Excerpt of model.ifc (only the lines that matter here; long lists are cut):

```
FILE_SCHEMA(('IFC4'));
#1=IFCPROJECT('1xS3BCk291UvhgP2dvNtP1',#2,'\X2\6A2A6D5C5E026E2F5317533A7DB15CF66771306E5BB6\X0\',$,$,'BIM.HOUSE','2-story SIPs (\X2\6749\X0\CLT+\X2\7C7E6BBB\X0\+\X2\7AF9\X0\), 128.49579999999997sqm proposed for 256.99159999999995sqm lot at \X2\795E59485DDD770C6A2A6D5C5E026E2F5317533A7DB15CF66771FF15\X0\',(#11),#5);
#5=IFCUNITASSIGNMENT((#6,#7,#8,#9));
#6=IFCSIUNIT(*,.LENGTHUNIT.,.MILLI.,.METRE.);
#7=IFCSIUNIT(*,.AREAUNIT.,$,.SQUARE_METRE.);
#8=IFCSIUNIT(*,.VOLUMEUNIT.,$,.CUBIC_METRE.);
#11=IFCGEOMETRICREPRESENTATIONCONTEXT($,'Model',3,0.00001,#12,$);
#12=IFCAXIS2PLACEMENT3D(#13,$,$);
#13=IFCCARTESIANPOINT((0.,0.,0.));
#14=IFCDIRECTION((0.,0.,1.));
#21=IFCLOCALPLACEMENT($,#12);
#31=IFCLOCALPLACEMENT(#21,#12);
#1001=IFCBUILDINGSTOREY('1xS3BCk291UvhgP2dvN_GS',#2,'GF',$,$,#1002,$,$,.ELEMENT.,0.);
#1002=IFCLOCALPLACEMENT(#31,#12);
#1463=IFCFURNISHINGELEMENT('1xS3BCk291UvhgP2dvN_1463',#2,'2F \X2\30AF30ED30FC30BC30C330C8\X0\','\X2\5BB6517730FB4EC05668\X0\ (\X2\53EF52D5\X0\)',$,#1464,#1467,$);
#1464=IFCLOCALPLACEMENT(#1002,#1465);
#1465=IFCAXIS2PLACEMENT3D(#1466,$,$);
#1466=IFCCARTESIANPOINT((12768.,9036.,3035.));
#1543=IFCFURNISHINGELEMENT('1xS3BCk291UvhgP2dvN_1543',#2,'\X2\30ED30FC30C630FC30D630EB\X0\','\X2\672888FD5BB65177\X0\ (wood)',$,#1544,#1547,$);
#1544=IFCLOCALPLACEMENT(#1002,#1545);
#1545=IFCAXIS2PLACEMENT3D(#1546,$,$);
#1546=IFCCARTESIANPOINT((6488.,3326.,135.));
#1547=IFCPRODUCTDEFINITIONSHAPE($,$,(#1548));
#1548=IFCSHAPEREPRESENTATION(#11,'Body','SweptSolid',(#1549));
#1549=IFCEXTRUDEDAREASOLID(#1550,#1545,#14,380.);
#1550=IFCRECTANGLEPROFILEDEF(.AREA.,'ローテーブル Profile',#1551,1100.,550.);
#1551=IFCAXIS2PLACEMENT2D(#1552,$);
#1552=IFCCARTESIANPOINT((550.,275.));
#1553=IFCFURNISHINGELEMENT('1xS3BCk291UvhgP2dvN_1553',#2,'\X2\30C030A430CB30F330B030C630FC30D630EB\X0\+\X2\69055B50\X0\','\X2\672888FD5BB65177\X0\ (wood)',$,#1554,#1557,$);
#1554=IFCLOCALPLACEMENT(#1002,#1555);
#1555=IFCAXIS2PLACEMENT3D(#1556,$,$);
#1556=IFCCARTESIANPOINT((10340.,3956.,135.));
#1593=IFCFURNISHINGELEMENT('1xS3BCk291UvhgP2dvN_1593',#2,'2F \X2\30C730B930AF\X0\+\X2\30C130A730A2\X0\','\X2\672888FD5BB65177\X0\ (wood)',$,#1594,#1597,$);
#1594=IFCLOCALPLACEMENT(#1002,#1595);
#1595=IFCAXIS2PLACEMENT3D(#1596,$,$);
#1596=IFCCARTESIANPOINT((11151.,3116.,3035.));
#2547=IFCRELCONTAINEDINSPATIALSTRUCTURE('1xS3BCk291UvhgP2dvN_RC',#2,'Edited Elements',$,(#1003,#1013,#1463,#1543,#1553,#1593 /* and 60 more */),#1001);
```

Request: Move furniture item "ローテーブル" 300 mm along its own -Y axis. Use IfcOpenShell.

```python
import ifcopenshell
import ifcopenshell.api.geometry
import ifcopenshell.util.placement
import ifcopenshell.util.unit

model = ifcopenshell.open("model.ifc")
unit_scale = ifcopenshell.util.unit.calculate_unit_scale(model)

item = model.by_id(1543)
matrix = ifcopenshell.util.placement.get_local_placement(item.ObjectPlacement)
matrix[:3, 3] -= matrix[:3, 1] * 0.3 / unit_scale
ifcopenshell.api.geometry.edit_object_placement(model, product=item, matrix=matrix, is_si=False)

print(ifcopenshell.util.placement.get_local_placement(item.ObjectPlacement).round(3) + 0.0)

model.write("model_rev.ifc")
```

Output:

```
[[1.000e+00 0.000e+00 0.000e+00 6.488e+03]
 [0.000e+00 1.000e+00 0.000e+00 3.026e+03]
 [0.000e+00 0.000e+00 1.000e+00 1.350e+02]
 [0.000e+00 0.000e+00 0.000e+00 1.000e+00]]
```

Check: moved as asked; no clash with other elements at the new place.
